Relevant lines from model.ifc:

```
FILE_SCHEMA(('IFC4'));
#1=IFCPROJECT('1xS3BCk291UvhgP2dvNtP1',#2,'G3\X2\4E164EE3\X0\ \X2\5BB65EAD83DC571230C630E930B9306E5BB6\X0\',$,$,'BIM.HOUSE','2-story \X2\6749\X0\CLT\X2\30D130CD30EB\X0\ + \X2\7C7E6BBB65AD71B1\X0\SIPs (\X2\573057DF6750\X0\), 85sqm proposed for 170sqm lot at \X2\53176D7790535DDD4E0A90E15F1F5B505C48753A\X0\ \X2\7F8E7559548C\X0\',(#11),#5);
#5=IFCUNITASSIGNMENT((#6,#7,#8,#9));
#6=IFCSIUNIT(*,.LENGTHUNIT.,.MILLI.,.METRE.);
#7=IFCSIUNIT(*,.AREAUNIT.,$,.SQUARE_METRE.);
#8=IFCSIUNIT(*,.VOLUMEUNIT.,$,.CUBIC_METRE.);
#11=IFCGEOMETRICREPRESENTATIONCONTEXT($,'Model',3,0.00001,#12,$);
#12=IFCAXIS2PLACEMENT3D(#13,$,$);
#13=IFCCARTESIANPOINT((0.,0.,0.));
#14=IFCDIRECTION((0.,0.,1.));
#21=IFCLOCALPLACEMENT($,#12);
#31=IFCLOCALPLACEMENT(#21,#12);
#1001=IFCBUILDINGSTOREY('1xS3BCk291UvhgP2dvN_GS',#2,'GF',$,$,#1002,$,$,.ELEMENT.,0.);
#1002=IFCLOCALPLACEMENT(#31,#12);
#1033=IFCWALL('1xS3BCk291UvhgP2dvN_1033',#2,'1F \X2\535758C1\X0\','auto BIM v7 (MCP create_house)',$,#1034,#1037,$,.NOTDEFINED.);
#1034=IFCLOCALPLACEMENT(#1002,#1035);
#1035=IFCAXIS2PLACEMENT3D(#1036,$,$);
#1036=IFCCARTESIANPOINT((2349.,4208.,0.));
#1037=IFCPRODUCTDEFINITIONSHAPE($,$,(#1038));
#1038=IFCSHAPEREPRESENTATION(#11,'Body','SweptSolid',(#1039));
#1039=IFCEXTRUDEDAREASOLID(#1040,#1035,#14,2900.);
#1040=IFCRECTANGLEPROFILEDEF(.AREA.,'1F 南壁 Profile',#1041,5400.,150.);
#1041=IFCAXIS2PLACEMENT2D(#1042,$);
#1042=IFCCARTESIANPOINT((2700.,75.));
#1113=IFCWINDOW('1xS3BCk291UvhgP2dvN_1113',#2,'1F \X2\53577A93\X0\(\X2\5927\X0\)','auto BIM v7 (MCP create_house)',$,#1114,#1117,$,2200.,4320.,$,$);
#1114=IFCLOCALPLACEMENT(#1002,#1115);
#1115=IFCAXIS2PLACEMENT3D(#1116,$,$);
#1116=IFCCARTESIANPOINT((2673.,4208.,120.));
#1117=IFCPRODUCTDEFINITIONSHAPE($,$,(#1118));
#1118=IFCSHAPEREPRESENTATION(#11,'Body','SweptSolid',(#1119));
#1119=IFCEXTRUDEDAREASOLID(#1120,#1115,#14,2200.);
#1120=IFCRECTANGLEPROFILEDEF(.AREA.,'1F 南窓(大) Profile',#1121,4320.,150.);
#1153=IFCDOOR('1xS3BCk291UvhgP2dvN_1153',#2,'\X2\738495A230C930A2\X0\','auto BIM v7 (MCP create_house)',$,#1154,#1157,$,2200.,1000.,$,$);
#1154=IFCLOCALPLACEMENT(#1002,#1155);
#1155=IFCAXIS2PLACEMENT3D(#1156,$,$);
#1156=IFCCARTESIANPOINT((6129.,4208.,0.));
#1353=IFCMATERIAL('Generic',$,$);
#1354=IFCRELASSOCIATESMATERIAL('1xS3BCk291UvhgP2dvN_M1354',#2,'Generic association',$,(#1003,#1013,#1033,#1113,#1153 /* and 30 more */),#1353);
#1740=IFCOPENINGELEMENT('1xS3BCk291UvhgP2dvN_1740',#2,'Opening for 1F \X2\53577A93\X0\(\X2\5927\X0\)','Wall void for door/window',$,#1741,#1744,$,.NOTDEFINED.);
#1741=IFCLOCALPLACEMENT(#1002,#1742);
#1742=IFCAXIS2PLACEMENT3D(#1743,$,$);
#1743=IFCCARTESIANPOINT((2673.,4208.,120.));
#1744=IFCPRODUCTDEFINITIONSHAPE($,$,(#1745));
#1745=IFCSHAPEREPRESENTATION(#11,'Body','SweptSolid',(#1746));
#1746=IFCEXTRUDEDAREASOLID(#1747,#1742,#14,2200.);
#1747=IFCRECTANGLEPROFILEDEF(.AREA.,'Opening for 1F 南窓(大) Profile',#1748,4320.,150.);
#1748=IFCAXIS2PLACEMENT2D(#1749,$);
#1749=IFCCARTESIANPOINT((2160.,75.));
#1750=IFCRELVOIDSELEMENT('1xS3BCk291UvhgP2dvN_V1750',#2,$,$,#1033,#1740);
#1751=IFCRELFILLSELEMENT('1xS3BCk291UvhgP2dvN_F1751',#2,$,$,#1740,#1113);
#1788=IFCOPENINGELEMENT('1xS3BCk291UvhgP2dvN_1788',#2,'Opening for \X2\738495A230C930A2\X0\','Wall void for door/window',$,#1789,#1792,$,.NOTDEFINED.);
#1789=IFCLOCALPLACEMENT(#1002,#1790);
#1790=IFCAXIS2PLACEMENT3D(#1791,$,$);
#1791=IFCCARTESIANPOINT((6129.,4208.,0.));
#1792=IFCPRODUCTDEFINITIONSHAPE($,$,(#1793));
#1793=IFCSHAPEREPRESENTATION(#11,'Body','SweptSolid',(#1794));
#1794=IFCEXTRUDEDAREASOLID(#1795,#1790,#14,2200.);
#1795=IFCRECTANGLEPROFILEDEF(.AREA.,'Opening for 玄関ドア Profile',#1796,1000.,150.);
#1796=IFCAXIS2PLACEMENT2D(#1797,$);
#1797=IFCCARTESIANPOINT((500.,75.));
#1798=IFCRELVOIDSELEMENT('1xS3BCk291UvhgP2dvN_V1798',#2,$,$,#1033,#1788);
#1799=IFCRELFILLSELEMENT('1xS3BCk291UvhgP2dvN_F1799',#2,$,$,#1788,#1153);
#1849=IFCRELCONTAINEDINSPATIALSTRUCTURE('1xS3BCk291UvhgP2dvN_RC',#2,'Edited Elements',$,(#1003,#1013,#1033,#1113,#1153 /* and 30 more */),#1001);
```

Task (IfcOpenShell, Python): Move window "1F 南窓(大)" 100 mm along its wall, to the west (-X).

```python
import ifcopenshell
import ifcopenshell.api.geometry
import ifcopenshell.util.placement
import ifcopenshell.util.unit

model = ifcopenshell.open("model.ifc")
unit_scale = ifcopenshell.util.unit.calculate_unit_scale(model)

window = model.by_id(1113)
opening = window.FillsVoids[0].RelatingOpeningElement
wall = opening.VoidsElements[0].RelatingBuildingElement

wall_matrix = ifcopenshell.util.placement.get_local_placement(wall.ObjectPlacement)
shift = wall_matrix[:3, 0] * -0.1 / unit_scale
before = ifcopenshell.util.placement.get_local_placement(window.ObjectPlacement)[:3, 3].copy()

# The window is not placed relative to its opening, so move both.
for product in (opening, window):
    matrix = ifcopenshell.util.placement.get_local_placement(product.ObjectPlacement)
    matrix[:3, 3] += shift
    ifcopenshell.api.geometry.edit_object_placement(model, product=product, matrix=matrix, is_si=False)

after = ifcopenshell.util.placement.get_local_placement(window.ObjectPlacement)[:3, 3]
print("window moved by", (after - before).round(3) + 0.0)

model.write("model_updated.ifc")
```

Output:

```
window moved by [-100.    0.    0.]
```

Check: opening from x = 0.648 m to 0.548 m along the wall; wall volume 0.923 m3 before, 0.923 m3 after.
